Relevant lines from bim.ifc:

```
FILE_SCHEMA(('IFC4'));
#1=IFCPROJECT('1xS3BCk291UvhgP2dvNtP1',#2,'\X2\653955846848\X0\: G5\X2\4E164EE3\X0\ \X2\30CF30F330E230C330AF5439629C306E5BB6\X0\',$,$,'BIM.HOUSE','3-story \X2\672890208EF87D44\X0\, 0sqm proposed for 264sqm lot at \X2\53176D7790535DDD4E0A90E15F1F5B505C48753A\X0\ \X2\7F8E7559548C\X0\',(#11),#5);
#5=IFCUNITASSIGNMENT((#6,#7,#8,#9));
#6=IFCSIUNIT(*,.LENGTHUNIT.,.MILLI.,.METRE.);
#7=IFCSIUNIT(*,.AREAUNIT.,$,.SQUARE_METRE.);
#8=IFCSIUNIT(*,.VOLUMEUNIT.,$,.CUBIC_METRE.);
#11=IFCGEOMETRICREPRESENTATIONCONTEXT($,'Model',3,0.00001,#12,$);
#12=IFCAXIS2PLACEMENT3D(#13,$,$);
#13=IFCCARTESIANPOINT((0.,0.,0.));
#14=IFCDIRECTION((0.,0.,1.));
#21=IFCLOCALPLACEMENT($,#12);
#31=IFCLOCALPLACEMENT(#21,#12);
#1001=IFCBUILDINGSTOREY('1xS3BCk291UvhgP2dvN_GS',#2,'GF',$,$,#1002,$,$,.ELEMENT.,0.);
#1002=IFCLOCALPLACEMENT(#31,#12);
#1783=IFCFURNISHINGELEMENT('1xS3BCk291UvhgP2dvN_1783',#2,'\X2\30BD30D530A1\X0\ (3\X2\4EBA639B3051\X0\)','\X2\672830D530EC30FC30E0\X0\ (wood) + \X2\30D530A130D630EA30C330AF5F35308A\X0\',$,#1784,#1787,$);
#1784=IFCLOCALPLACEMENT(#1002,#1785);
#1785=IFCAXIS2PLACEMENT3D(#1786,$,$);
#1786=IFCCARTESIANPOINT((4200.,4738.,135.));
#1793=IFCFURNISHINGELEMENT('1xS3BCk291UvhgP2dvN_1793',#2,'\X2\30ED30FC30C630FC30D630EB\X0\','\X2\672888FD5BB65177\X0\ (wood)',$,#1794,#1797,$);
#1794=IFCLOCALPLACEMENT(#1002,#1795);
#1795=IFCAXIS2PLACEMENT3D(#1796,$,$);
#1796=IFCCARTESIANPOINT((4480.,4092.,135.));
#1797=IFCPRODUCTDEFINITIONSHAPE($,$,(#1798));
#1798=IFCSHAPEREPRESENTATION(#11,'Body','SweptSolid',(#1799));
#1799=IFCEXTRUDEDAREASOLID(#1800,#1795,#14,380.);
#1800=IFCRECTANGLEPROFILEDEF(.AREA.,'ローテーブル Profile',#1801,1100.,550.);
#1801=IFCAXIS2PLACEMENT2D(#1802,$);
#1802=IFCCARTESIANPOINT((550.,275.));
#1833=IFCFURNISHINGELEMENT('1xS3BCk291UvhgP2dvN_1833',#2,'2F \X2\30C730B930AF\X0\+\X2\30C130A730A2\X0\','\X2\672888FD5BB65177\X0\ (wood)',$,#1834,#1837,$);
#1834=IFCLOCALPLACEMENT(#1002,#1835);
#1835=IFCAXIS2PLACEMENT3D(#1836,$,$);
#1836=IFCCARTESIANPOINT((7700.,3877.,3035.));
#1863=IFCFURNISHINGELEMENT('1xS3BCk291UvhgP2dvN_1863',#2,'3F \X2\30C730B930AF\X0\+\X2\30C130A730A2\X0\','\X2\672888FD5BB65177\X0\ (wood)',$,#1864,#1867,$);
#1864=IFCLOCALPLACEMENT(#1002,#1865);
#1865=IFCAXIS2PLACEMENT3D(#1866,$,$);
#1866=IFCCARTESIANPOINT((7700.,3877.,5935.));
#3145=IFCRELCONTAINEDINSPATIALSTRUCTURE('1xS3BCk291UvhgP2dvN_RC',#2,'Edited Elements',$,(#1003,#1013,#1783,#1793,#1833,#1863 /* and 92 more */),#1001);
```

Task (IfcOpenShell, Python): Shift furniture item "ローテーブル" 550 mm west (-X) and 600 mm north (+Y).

```python
import ifcopenshell
import ifcopenshell.api.geometry
import ifcopenshell.util.placement
import ifcopenshell.util.unit

model = ifcopenshell.open("bim.ifc")
unit_scale = ifcopenshell.util.unit.calculate_unit_scale(model)

item = model.by_guid("1xS3BCk291UvhgP2dvN_1793")
matrix = ifcopenshell.util.placement.get_local_placement(item.ObjectPlacement)
matrix[0, 3] -= 0.55 / unit_scale
matrix[1, 3] += 0.6 / unit_scale
ifcopenshell.api.geometry.edit_object_placement(model, product=item, matrix=matrix, is_si=False)

print(ifcopenshell.util.placement.get_local_placement(item.ObjectPlacement).round(3) + 0.0)

model.write("bim_updated.ifc")
```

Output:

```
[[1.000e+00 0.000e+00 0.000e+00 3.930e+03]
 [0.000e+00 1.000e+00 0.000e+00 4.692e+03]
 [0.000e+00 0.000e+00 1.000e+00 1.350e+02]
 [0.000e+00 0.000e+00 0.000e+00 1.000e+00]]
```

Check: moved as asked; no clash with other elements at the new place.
